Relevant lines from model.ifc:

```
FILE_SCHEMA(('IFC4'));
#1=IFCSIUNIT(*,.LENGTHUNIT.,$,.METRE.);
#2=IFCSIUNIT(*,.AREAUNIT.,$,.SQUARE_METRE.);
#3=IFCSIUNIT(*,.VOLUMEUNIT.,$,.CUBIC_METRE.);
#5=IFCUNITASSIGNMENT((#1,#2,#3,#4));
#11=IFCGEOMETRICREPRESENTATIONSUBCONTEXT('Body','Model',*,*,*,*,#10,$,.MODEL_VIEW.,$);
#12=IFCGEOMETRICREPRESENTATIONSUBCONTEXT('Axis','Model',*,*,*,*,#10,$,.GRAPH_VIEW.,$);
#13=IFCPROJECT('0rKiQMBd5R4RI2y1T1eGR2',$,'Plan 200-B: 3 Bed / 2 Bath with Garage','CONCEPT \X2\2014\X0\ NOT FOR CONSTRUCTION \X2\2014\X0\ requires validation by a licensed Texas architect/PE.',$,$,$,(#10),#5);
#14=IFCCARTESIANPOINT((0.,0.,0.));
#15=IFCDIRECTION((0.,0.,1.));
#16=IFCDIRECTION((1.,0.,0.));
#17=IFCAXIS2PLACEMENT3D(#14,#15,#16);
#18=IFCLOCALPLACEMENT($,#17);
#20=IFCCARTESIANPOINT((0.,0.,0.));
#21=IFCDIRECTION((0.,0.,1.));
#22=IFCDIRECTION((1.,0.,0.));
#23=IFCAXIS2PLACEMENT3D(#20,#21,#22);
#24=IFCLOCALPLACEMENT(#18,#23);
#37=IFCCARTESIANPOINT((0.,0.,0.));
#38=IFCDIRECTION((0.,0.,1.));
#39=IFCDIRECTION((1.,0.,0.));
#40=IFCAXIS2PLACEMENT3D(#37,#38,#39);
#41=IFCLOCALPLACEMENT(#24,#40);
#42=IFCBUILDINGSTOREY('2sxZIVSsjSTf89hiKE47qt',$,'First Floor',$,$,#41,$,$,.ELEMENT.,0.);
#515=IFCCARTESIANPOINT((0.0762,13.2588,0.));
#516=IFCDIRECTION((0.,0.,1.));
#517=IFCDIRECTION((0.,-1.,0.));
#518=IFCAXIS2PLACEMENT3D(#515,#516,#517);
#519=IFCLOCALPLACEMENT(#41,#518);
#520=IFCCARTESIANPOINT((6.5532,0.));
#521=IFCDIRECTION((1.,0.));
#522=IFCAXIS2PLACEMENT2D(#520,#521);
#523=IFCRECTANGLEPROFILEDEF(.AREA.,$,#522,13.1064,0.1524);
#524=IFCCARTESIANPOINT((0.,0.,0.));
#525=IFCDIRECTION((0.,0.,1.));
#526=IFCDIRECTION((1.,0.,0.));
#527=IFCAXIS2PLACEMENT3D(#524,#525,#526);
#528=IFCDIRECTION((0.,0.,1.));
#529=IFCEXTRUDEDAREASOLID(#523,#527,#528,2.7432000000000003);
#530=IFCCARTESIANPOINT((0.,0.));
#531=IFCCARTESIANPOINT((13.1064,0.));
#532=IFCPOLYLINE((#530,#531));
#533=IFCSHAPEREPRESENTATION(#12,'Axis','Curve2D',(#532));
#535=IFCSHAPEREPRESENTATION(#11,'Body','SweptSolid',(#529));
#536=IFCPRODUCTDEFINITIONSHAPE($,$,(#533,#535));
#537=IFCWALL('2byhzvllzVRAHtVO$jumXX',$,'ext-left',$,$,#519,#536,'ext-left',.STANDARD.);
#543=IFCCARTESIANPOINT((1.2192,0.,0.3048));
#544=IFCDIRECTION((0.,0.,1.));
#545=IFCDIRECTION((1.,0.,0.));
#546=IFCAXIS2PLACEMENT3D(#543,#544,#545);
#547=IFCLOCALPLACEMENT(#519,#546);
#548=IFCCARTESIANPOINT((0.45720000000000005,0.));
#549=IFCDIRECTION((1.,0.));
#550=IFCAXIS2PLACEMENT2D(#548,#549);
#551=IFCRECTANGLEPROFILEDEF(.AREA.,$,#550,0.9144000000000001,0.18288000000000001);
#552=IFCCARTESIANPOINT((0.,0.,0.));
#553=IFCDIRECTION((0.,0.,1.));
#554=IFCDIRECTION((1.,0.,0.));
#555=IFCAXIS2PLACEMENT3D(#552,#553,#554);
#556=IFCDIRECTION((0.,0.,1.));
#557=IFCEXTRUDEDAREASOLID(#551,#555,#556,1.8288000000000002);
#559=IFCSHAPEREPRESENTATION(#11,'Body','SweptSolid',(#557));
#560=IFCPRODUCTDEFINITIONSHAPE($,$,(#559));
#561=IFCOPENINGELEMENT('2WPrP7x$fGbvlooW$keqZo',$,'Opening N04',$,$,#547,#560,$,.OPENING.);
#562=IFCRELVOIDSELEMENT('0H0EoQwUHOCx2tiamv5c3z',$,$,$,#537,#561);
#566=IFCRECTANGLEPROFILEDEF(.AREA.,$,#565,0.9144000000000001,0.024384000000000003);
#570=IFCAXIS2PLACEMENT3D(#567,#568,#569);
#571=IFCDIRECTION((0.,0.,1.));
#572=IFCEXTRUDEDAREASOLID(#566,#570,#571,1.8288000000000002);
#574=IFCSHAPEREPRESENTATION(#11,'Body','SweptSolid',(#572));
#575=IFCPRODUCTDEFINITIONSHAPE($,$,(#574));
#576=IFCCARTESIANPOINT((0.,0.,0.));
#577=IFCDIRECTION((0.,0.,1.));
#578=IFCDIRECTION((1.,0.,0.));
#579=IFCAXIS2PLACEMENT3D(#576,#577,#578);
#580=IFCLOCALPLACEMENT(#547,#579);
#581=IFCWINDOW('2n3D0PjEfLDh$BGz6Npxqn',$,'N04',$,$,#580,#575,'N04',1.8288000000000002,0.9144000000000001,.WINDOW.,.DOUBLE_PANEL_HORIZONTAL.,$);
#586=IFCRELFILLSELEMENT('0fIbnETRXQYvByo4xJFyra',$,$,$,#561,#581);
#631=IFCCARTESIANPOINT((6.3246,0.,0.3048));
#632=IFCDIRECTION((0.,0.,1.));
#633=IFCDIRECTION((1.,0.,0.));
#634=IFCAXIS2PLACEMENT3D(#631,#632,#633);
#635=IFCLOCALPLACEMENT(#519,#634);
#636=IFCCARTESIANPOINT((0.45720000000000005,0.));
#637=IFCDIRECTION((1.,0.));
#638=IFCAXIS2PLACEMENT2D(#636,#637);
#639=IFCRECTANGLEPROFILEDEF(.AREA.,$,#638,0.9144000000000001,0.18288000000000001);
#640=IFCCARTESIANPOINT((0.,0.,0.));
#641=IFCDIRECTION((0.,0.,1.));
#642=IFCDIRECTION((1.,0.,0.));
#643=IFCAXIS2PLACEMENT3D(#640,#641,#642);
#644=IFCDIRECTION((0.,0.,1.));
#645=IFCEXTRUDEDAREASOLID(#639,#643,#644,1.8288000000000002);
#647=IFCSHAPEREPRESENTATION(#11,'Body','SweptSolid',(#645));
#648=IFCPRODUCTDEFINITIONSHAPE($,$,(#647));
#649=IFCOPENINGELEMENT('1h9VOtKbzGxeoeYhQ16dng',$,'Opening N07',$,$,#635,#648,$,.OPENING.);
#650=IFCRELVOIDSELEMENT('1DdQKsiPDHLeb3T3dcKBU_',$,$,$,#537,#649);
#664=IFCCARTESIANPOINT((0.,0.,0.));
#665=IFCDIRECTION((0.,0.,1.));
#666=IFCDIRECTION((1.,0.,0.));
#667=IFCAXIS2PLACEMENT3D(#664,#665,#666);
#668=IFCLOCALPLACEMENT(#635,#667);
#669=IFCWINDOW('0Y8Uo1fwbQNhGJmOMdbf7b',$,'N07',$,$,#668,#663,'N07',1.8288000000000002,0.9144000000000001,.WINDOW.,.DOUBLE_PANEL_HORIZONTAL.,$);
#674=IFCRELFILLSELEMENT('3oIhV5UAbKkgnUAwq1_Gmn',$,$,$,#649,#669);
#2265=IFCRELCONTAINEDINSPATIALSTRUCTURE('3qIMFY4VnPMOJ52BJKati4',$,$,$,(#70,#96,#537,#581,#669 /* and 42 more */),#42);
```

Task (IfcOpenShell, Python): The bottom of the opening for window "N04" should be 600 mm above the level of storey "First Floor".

```python
import numpy as np
import ifcopenshell
import ifcopenshell.api.geometry
import ifcopenshell.geom
import ifcopenshell.util.element
import ifcopenshell.util.placement
import ifcopenshell.util.shape
import ifcopenshell.util.unit

model = ifcopenshell.open("model.ifc")
unit_scale = ifcopenshell.util.unit.calculate_unit_scale(model)

window = model.by_guid("2n3D0PjEfLDh$BGz6Npxqn")
opening = window.FillsVoids[0].RelatingOpeningElement
storey = ifcopenshell.util.element.get_container(window, ifc_class="IfcBuildingStorey")
level = ifcopenshell.util.placement.get_local_placement(storey.ObjectPlacement)[2, 3]

# The opening's origin need not be at the sill, so measure its lowest point.
shape = ifcopenshell.geom.create_shape(ifcopenshell.geom.settings(), opening)
bottom = ifcopenshell.util.shape.get_shape_bottom_elevation(shape, shape.geometry) / unit_scale
dz = level + 0.6 / unit_scale - bottom

shift = np.array([0.0, 0.0, dz])
# The window is placed relative to its opening, so it follows when the opening moves.
matrix = ifcopenshell.util.placement.get_local_placement(opening.ObjectPlacement)
matrix[:3, 3] += shift
ifcopenshell.api.geometry.edit_object_placement(
    model, product=opening, matrix=matrix, is_si=False, should_transform_children=True
)

print(f"moved by {dz * unit_scale:+.3f} m")

model.write("model_updated.ifc")
```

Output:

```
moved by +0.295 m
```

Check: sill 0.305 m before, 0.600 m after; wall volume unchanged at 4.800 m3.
